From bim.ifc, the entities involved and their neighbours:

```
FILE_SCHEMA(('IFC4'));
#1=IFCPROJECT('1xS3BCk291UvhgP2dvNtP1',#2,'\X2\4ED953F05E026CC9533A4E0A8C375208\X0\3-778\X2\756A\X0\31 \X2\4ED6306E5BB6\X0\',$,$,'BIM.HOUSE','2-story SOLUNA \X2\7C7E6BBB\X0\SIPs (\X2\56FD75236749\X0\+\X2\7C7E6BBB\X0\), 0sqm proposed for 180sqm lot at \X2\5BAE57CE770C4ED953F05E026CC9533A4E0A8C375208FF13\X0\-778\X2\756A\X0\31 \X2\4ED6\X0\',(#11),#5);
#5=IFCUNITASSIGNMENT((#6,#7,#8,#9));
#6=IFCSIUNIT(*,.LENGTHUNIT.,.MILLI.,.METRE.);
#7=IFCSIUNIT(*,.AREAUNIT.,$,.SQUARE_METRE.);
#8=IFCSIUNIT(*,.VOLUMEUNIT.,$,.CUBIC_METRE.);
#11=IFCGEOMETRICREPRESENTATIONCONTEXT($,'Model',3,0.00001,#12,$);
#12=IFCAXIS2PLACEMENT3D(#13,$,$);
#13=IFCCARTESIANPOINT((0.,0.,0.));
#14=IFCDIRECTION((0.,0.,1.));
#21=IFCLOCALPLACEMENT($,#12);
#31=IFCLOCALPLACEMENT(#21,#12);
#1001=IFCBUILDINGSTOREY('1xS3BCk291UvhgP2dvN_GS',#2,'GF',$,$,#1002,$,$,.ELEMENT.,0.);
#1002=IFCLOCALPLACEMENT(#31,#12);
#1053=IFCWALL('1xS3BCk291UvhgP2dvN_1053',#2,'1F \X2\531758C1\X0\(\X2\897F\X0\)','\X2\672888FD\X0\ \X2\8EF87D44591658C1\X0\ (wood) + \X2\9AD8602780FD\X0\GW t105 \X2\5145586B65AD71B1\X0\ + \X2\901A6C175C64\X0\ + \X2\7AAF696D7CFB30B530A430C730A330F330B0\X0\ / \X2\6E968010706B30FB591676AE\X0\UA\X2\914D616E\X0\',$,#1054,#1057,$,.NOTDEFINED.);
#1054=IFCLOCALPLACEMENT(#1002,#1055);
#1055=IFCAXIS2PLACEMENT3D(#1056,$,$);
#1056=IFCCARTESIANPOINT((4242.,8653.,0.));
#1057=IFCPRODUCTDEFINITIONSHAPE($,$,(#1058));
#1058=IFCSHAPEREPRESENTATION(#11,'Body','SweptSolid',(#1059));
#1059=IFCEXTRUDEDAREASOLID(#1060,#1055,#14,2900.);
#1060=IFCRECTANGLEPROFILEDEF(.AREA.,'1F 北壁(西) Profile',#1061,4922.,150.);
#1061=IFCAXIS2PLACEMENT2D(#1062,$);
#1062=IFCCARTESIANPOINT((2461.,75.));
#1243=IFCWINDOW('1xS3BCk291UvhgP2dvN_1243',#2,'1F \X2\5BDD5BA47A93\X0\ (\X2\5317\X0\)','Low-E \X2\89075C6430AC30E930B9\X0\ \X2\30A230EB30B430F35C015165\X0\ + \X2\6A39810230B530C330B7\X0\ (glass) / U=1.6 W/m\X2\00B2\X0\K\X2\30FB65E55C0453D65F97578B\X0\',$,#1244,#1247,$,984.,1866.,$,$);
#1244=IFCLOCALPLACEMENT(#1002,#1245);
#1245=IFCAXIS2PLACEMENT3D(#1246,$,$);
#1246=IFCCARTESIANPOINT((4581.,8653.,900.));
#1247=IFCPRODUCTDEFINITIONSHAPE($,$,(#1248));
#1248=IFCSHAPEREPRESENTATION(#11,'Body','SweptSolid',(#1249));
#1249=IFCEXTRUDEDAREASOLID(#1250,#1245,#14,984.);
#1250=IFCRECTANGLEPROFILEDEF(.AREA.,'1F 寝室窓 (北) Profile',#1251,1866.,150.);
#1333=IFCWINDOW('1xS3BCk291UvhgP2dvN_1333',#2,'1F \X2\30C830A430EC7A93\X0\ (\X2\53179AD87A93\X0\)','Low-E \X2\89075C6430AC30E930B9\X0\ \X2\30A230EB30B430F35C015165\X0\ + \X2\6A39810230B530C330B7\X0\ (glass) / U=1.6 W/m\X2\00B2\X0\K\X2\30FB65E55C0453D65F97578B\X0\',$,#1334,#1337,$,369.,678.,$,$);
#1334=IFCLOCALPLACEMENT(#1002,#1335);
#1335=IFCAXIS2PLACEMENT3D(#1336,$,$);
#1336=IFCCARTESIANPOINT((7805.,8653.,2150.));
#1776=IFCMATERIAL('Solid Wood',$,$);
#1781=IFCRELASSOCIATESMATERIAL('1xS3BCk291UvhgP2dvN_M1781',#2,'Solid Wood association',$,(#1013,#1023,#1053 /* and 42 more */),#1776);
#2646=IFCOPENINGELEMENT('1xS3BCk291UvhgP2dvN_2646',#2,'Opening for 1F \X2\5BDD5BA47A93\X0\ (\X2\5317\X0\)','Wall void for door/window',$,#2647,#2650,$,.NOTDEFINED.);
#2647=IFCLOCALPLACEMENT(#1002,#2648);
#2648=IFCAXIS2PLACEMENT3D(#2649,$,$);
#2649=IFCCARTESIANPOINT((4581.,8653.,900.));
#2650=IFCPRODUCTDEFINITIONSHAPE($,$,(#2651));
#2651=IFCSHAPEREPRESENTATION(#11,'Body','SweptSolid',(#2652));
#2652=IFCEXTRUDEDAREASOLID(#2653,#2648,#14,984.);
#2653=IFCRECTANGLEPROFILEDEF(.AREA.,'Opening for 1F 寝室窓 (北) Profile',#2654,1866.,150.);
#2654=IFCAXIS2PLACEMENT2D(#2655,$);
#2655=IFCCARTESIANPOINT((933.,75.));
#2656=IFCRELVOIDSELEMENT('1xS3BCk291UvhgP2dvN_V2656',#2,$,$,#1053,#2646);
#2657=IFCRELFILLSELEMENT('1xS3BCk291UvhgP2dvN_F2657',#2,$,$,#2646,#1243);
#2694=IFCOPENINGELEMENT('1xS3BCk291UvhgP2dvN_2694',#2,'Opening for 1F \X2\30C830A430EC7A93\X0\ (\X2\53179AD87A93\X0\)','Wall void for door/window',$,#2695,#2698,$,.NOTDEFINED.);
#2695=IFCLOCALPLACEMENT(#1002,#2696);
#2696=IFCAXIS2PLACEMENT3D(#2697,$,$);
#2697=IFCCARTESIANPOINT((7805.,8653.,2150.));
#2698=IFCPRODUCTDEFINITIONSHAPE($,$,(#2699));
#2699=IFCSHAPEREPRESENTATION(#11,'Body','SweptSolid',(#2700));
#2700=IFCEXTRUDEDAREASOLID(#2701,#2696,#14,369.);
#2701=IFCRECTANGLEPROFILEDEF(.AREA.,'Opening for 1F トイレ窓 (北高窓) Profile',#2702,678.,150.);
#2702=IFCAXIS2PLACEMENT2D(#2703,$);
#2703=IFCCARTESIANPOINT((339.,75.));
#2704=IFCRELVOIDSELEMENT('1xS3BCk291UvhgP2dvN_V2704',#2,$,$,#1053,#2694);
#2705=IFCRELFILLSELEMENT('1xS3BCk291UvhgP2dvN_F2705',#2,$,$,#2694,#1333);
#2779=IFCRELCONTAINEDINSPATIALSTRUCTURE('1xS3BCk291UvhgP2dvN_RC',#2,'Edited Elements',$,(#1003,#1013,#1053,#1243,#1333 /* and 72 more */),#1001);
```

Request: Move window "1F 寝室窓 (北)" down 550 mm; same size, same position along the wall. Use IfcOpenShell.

```python
import numpy as np
import ifcopenshell
import ifcopenshell.api.geometry
import ifcopenshell.util.placement
import ifcopenshell.util.unit

model = ifcopenshell.open("bim.ifc")
unit_scale = ifcopenshell.util.unit.calculate_unit_scale(model)

window = model.by_guid("1xS3BCk291UvhgP2dvN_1243")
opening = window.FillsVoids[0].RelatingOpeningElement
dz = -0.55 / unit_scale

shift = np.array([0.0, 0.0, dz])
# The window is not placed relative to its opening, so move both.
for product in (opening, window):
    matrix = ifcopenshell.util.placement.get_local_placement(product.ObjectPlacement)
    matrix[:3, 3] += shift
    ifcopenshell.api.geometry.edit_object_placement(model, product=product, matrix=matrix, is_si=False)

print(f"moved by {dz * unit_scale:+.3f} m")

model.write("bim_updated.ifc")
```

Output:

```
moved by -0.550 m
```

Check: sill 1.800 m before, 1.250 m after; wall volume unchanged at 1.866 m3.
